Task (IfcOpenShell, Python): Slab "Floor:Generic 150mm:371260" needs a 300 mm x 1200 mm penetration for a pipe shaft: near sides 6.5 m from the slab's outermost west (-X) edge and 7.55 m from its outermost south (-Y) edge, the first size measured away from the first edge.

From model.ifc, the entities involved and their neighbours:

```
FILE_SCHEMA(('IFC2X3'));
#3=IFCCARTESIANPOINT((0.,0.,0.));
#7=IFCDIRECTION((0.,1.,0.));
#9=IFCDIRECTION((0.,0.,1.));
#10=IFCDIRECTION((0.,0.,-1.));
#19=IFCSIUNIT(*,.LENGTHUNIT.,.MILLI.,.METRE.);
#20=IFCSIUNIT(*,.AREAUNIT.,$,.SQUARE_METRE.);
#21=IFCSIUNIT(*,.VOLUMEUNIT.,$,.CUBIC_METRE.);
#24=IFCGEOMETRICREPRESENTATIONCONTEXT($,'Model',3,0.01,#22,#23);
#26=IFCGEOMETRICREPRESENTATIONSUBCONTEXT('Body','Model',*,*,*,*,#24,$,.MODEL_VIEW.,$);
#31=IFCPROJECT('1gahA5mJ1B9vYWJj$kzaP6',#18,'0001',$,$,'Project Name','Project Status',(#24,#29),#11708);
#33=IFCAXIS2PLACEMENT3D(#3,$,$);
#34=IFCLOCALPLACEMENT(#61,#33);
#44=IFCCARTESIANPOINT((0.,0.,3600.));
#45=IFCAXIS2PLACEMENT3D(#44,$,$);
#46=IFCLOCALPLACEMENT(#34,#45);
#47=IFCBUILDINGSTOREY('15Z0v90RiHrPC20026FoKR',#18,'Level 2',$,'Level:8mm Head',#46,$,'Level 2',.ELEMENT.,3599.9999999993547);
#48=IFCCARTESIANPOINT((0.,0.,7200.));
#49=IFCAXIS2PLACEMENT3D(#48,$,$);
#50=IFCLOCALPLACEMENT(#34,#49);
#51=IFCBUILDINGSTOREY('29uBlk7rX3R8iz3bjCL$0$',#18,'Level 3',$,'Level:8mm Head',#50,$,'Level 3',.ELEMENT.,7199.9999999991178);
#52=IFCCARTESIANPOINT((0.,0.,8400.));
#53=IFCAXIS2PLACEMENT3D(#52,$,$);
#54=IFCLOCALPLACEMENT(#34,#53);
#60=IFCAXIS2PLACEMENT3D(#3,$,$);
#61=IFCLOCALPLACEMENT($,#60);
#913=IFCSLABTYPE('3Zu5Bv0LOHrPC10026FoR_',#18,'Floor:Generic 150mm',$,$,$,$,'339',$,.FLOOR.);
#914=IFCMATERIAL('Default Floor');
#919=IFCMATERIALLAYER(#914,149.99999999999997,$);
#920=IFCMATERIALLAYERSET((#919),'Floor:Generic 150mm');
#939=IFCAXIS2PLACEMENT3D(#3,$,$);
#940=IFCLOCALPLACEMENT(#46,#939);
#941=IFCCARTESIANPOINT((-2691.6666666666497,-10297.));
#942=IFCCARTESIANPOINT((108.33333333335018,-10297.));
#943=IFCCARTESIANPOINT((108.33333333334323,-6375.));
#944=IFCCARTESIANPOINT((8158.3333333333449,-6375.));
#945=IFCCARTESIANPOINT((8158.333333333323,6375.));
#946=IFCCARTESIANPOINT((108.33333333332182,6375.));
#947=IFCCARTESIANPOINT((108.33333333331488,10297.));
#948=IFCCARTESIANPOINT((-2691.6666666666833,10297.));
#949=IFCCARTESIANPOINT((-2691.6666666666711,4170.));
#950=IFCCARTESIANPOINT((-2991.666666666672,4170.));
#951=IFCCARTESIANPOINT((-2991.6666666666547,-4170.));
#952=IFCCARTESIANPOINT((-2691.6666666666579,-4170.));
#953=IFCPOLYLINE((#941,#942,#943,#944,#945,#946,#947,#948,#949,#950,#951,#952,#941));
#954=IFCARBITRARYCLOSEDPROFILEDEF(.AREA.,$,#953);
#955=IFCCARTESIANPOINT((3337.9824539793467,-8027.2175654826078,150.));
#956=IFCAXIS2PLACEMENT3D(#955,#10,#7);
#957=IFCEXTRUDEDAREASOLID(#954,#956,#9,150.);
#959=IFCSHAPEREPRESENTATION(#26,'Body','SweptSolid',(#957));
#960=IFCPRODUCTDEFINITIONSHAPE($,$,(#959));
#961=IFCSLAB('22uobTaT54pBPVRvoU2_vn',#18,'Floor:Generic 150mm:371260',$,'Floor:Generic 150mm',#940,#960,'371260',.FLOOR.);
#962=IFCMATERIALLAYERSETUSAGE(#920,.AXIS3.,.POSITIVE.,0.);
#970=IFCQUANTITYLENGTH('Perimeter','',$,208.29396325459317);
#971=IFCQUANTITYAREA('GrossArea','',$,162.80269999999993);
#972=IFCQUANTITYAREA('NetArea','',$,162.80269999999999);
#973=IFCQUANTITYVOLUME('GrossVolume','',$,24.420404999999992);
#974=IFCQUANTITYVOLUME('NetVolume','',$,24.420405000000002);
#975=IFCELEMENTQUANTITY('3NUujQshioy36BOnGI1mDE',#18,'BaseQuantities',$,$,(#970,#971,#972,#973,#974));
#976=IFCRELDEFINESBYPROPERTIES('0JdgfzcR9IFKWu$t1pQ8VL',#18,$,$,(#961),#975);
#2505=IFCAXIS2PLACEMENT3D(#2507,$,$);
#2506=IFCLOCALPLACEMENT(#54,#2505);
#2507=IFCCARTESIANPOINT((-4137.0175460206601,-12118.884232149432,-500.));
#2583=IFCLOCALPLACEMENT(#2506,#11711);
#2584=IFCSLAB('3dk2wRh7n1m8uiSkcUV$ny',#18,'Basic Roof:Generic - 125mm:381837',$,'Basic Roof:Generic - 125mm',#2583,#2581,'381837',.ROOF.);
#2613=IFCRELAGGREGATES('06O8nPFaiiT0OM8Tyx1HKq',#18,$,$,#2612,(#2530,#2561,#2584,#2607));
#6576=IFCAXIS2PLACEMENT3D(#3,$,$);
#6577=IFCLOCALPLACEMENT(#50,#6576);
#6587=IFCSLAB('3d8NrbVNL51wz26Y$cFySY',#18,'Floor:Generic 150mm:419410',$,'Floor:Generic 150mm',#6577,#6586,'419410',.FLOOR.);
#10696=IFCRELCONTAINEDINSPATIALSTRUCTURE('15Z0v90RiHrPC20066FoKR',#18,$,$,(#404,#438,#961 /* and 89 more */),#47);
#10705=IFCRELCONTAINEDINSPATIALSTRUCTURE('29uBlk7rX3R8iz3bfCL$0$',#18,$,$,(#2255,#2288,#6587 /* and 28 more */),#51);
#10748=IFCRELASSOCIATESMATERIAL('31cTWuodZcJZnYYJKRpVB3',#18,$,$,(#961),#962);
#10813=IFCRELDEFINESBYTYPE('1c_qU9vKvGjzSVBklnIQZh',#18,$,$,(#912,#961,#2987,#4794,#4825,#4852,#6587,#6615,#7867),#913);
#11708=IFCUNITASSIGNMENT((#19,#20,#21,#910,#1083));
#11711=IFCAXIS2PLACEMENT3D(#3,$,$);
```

```python
import numpy as np
import ifcopenshell
import ifcopenshell.api.feature
import ifcopenshell.api.geometry
import ifcopenshell.api.pset
import ifcopenshell.api.root
import ifcopenshell.geom
import ifcopenshell.util.element
import ifcopenshell.util.placement
import ifcopenshell.util.representation
import ifcopenshell.util.shape
import ifcopenshell.util.unit

model = ifcopenshell.open("model.ifc")
unit_scale = ifcopenshell.util.unit.calculate_unit_scale(model)
area_scale = ifcopenshell.util.unit.calculate_unit_scale(model, "AREAUNIT")
volume_scale = ifcopenshell.util.unit.calculate_unit_scale(model, "VOLUMEUNIT")
settings = ifcopenshell.geom.settings()


def volume(element):
    """Net volume in cubic metres, openings subtracted."""
    shape = ifcopenshell.geom.create_shape(settings, element)
    return ifcopenshell.util.shape.get_volume(shape.geometry)


slab = model.by_guid("22uobTaT54pBPVRvoU2_vn")
before = volume(slab)

# Extent in the slab's own axes, in metres. The edges named are its -X and -Y sides.
slab_shape = ifcopenshell.geom.create_shape(settings, slab)
vertices = ifcopenshell.util.shape.get_vertices(slab_shape.geometry)
x_min, y_min, bottom = vertices.min(axis=0)
top = vertices[:, 2].max()

opening = ifcopenshell.api.root.create_entity(model, ifc_class="IfcOpeningElement", name="Pipe shaft opening")
context = ifcopenshell.util.representation.get_context(model, "Model", "Body", "MODEL_VIEW")
width, depth = 0.3, 1.2
outline = [(0.0, 0.0), (width, 0.0), (width, depth), (0.0, depth), (0.0, 0.0)]
# Overshoot both faces by 50 mm so the cut is clean.
shape = ifcopenshell.api.geometry.add_slab_representation(
    model, context=context, depth=top - bottom + 0.1, polyline=outline
)
ifcopenshell.api.geometry.assign_representation(model, product=opening, representation=shape)

matrix = ifcopenshell.util.placement.get_local_placement(slab.ObjectPlacement)
matrix[:, 3] = matrix @ np.append(np.array([x_min + 6.5, y_min + 7.55, bottom - 0.05]) / unit_scale, 1.0)
ifcopenshell.api.geometry.edit_object_placement(model, product=opening, matrix=matrix, is_si=False)
ifcopenshell.api.feature.add_feature(model, feature=opening, element=slab)

after = volume(slab)

# Update the slab's stored quantities.
qto = model.by_id(ifcopenshell.util.element.get_pset(slab, "BaseQuantities", should_inherit=False)["id"])
ifcopenshell.api.pset.edit_qto(model, qto=qto, properties={
    "NetArea": after / (top - bottom) / area_scale,
    "NetVolume": after / volume_scale,
})

print(f"slab volume {before:.3f} -> {after:.3f} m3")

model.write("model_v2.ifc")
```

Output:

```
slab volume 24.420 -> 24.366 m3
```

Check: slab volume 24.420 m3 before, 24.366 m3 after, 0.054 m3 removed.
